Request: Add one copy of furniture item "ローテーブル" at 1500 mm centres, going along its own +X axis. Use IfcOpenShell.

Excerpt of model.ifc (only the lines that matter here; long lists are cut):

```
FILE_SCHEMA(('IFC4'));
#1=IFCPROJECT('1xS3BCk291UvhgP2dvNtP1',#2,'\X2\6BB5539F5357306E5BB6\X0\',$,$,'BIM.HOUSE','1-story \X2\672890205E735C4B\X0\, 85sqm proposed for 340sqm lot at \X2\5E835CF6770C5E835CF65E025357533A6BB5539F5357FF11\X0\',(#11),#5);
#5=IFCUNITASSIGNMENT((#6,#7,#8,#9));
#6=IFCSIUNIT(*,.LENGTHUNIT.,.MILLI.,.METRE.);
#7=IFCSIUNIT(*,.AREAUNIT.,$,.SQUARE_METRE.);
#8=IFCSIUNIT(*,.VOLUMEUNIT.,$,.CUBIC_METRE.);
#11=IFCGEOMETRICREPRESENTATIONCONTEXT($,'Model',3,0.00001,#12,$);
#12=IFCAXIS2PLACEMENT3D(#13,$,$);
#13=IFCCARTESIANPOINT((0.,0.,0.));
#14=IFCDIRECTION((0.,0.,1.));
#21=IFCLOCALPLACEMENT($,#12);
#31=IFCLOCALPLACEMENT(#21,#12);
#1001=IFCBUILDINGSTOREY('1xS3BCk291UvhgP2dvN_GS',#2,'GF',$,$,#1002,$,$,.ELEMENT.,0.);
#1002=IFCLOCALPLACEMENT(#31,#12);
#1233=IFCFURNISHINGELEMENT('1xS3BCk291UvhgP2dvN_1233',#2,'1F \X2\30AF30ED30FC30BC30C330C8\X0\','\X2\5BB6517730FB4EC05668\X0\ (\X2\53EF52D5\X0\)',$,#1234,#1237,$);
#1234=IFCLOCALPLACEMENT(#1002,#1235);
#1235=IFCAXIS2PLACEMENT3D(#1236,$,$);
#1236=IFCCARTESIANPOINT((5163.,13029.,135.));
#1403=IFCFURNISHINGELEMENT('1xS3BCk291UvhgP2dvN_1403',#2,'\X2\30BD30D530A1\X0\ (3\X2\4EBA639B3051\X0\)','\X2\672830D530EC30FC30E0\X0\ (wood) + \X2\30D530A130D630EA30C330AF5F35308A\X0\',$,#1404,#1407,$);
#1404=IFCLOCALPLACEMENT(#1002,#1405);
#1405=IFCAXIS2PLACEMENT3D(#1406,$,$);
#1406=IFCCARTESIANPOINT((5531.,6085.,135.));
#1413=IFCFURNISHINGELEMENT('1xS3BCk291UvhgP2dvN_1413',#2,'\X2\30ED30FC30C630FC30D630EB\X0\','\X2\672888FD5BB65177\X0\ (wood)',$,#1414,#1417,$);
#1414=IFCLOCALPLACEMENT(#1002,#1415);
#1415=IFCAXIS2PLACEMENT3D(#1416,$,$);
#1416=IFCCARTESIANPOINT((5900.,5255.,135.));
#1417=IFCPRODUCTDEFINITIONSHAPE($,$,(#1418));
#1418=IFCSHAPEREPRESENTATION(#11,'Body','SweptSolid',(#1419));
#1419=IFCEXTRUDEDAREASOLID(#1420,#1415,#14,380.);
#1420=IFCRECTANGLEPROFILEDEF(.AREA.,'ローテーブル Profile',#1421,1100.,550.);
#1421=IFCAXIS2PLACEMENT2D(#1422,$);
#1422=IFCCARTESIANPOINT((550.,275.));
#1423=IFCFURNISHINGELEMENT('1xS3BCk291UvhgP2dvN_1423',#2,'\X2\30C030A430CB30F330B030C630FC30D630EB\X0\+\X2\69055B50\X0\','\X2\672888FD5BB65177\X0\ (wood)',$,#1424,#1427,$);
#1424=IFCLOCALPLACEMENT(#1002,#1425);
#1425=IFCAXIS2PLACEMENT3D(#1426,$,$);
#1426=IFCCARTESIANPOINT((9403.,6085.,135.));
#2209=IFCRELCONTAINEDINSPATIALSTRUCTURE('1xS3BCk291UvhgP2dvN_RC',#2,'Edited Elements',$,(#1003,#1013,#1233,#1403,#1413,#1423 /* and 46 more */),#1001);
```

```python
import ifcopenshell
import ifcopenshell.api.geometry
import ifcopenshell.api.root
import ifcopenshell.util.element
import ifcopenshell.util.placement

model = ifcopenshell.open("model.ifc")


def reuse_history(source, copy):
    """copy_class also copies each property set's owner history, people and application; keep the originals."""
    for rel in copy.IsDefinedBy:
        if rel.is_a("IfcRelDefinesByProperties") and (history := rel.RelatingPropertyDefinition.OwnerHistory):
            rel.RelatingPropertyDefinition.OwnerHistory = source.OwnerHistory
            ifcopenshell.util.element.remove_deep2(model, history)


source = model.by_guid("1xS3BCk291UvhgP2dvN_1413")
base = ifcopenshell.util.placement.get_local_placement(source.ObjectPlacement)
step = base[:3, 0] * 1500.0

for i in range(1, 2):
    copy = ifcopenshell.api.root.copy_class(model, product=source)
    copy.Representation = ifcopenshell.util.element.copy_deep(
        model, source.Representation, exclude=["IfcGeometricRepresentationContext", "IfcRepresentationMap"]
    )
    reuse_history(source, copy)
    matrix = base.copy()
    matrix[:3, 3] += i * step
    print("added at", matrix[:3, 3].round(3) + 0.0)
    ifcopenshell.api.geometry.edit_object_placement(model, product=copy, matrix=matrix, is_si=False)

model.write("model_v2.ifc")
```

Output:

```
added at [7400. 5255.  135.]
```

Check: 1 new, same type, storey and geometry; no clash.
